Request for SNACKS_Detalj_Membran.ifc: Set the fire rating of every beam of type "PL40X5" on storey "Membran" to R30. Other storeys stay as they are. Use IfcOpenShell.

First a look at what the model holds.

```python
import ifcopenshell
import ifcopenshell.util.element

model = ifcopenshell.open("SNACKS_Detalj_Membran.ifc")
print(model.schema)
storey = next(s for s in model.by_type("IfcBuildingStorey") if s.Name == "Membran")
beams = [e for e in ifcopenshell.util.element.get_decomposition(storey) if e.is_a("IfcBeam")]
seen = {}
for e in beams:
    element_type = ifcopenshell.util.element.get_type(e)
    key = (element_type.Name if element_type != e and element_type else None, ifcopenshell.util.element.get_pset(e, "Pset_BeamCommon", "FireRating"))
    seen[key] = seen.get(key, 0) + 1
for (name, value), count in sorted(seen.items(), key=str):
    print(count, "x", name, "|", value)
```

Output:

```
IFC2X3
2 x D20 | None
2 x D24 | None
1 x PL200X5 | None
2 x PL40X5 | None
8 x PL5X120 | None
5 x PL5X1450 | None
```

```python
import ifcopenshell
import ifcopenshell.api.pset
import ifcopenshell.util.element

model = ifcopenshell.open("SNACKS_Detalj_Membran.ifc")

storey = next(s for s in model.by_type("IfcBuildingStorey") if s.Name == "Membran")
beams = [e for e in ifcopenshell.util.element.get_decomposition(storey) if e.is_a("IfcBeam")]

count = 0
for e in beams:
    element_type = ifcopenshell.util.element.get_type(e)
    if element_type in (None, e) or element_type.Name != "PL40X5":
        continue
    # add_pset returns the element's existing set when there is one.
    pset = ifcopenshell.api.pset.add_pset(model, product=e, name="Pset_BeamCommon")
    ifcopenshell.api.pset.edit_pset(model, pset=pset, properties={"FireRating": "R30"})
    count += 1

print(count, "beams updated")

model.write("SNACKS_Detalj_Membran-out.ifc")
```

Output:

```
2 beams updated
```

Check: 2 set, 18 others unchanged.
